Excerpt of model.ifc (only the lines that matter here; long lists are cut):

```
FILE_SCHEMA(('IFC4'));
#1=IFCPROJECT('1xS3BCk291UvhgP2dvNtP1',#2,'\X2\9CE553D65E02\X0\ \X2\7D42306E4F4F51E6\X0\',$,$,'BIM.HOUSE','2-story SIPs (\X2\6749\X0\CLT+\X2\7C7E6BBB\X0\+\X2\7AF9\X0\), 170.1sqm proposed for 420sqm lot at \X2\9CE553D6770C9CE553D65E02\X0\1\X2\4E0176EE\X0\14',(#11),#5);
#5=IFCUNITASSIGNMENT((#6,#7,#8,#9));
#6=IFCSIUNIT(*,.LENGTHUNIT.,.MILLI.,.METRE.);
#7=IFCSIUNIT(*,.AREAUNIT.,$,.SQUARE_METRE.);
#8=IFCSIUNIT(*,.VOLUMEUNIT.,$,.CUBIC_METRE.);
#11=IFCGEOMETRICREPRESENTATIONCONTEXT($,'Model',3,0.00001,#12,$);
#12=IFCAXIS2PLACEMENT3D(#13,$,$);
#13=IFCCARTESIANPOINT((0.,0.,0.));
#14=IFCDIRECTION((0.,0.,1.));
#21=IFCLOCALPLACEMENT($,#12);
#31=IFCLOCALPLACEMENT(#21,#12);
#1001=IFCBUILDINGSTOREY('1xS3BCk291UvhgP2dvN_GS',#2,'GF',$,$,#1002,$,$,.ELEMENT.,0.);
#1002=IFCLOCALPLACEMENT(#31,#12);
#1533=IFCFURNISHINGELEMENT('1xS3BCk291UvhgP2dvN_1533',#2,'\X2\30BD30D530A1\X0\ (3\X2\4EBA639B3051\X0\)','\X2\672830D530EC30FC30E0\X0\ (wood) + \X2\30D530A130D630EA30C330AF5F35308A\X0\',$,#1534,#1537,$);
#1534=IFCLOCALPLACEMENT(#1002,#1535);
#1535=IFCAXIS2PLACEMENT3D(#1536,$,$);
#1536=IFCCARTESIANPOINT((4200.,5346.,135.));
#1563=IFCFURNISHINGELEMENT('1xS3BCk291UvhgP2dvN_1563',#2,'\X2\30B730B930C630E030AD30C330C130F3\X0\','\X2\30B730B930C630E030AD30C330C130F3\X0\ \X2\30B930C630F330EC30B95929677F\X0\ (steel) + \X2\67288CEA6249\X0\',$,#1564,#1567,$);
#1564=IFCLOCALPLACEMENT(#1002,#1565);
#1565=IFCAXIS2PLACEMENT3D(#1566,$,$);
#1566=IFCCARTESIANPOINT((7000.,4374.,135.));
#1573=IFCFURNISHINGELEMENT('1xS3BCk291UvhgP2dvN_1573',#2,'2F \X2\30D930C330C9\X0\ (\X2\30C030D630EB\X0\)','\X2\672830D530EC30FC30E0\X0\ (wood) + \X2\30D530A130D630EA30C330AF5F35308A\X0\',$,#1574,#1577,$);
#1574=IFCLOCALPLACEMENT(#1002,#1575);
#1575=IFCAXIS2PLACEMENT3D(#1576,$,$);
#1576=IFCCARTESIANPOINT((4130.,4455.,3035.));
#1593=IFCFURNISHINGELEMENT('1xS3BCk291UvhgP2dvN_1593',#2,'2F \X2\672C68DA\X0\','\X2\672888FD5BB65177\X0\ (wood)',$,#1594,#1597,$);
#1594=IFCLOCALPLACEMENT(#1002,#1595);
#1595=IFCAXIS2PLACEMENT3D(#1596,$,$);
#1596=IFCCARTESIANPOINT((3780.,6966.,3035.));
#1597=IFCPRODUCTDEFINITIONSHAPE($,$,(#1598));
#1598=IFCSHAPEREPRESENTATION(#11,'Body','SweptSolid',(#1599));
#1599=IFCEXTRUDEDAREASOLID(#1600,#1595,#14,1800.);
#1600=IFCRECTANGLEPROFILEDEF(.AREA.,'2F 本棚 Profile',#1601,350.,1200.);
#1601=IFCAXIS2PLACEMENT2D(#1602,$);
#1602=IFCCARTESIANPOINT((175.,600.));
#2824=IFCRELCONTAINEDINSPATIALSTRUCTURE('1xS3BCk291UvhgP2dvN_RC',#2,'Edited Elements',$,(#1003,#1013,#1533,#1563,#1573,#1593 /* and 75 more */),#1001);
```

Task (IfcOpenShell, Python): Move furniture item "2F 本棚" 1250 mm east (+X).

```python
import ifcopenshell
import ifcopenshell.api.geometry
import ifcopenshell.util.placement
import ifcopenshell.util.unit

model = ifcopenshell.open("model.ifc")
unit_scale = ifcopenshell.util.unit.calculate_unit_scale(model)

item = model.by_guid("1xS3BCk291UvhgP2dvN_1593")
matrix = ifcopenshell.util.placement.get_local_placement(item.ObjectPlacement)
matrix[0, 3] += 1.25 / unit_scale
ifcopenshell.api.geometry.edit_object_placement(model, product=item, matrix=matrix, is_si=False)

print(ifcopenshell.util.placement.get_local_placement(item.ObjectPlacement).round(3) + 0.0)

model.write("model-out.ifc")
```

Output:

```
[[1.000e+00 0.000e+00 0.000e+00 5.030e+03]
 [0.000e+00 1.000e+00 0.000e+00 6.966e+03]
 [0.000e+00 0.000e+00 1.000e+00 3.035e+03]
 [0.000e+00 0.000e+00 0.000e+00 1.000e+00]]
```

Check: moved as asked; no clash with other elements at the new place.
